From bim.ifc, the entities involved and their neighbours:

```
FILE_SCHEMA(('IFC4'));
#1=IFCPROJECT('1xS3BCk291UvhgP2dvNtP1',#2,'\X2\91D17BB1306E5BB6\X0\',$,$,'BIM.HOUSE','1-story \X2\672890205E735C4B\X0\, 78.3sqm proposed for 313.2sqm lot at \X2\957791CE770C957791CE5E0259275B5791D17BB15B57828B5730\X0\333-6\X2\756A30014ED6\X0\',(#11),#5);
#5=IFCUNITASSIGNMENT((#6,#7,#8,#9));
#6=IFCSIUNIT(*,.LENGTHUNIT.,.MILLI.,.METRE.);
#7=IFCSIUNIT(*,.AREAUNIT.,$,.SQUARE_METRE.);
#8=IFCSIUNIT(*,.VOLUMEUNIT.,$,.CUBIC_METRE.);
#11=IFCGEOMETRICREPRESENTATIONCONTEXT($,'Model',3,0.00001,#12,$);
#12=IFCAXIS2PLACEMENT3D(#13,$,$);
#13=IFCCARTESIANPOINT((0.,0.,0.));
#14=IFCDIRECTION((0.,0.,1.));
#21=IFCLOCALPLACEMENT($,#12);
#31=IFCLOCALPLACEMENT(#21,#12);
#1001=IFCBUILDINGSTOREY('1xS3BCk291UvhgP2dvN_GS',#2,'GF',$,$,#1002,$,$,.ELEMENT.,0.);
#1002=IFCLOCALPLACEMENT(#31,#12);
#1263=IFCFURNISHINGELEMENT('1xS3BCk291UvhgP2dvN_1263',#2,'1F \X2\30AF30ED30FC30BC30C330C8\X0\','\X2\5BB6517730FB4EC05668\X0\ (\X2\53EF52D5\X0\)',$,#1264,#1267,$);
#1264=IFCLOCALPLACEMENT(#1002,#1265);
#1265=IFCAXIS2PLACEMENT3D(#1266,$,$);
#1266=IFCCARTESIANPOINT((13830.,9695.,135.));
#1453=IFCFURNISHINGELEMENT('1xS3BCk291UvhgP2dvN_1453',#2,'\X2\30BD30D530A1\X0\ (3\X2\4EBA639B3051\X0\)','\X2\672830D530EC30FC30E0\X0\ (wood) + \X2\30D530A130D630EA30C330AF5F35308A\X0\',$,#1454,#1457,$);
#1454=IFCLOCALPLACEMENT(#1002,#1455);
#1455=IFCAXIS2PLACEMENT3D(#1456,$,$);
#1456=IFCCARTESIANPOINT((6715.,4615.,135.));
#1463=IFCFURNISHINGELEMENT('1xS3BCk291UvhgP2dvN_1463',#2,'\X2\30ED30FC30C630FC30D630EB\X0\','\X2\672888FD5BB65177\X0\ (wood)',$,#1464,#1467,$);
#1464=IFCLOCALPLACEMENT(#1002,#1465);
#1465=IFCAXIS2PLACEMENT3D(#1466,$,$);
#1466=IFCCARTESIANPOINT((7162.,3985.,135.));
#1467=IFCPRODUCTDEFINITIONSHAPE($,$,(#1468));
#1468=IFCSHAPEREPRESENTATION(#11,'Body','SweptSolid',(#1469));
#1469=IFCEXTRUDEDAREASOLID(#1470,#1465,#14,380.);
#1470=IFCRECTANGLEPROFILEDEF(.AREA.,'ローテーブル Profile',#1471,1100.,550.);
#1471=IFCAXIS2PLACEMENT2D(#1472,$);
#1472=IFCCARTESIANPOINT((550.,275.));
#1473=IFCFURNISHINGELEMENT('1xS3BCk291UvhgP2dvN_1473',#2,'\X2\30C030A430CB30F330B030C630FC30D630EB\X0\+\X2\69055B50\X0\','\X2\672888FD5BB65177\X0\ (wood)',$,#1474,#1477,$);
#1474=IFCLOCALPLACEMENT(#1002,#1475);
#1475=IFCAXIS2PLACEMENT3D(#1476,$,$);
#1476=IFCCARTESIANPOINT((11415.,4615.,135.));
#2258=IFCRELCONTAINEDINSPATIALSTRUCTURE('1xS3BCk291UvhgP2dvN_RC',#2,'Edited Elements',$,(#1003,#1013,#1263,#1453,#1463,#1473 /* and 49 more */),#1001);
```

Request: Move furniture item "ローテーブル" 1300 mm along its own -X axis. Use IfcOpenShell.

```python
import ifcopenshell
import ifcopenshell.api.geometry
import ifcopenshell.util.placement

model = ifcopenshell.open("bim.ifc")

item = model.by_guid("1xS3BCk291UvhgP2dvN_1463")
matrix = ifcopenshell.util.placement.get_local_placement(item.ObjectPlacement)
matrix[:3, 3] -= matrix[:3, 0] * 1300.0
ifcopenshell.api.geometry.edit_object_placement(model, product=item, matrix=matrix, is_si=False)

print(ifcopenshell.util.placement.get_local_placement(item.ObjectPlacement).round(3) + 0.0)

model.write("bim_edited.ifc")
```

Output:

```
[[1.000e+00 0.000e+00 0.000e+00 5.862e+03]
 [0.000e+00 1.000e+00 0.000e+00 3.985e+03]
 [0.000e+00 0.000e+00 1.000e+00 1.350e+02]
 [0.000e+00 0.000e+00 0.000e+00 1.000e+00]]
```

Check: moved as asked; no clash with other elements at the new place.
